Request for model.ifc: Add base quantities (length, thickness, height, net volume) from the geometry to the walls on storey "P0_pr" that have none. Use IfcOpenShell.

First a look at what the model holds.

```python
import ifcopenshell
import ifcopenshell.util.element
import ifcopenshell.util.unit

model = ifcopenshell.open("model.ifc")
print(model.schema)
for unit_type in ("LENGTHUNIT", "AREAUNIT", "VOLUMEUNIT"):
    print(unit_type, ifcopenshell.util.unit.calculate_unit_scale(model, unit_type))
storey = next(s for s in model.by_type("IfcBuildingStorey") if s.Name == "P0_pr")
walls = [e for e in ifcopenshell.util.element.get_decomposition(storey) if e.is_a("IfcWall")]
for e in sorted(walls, key=lambda e: e.id()):
    print(e.id(), e.is_a(), e.Name, list(ifcopenshell.util.element.get_psets(e, qtos_only=True)), sep=" | ")
```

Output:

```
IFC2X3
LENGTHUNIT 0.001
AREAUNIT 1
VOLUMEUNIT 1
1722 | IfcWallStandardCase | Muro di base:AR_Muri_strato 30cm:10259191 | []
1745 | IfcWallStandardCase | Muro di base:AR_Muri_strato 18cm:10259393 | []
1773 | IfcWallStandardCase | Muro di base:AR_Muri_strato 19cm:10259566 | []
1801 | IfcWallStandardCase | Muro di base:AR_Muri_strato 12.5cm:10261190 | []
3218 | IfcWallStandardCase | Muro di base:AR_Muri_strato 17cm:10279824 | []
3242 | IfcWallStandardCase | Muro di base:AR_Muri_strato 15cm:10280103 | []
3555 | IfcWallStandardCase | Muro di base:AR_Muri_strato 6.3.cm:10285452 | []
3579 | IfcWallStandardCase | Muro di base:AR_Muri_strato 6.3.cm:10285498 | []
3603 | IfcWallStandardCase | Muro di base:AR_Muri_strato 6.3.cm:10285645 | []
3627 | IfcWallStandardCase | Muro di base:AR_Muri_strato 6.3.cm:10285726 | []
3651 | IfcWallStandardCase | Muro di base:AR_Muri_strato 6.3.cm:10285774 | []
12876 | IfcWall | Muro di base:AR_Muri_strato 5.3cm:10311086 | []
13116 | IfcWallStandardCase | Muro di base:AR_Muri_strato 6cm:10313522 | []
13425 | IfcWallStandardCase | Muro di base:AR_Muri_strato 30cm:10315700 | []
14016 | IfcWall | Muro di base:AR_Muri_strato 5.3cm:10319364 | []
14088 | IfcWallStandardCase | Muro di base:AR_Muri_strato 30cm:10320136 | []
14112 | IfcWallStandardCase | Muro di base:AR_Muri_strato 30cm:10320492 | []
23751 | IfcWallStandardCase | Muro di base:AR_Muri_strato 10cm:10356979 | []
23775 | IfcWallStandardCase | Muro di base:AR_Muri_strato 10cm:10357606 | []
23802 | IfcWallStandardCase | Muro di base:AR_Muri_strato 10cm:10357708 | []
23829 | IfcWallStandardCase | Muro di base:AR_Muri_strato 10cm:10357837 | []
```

```python
import ifcopenshell
import ifcopenshell.api.pset
import ifcopenshell.geom
import ifcopenshell.util.element
import ifcopenshell.util.shape
import ifcopenshell.util.unit

model = ifcopenshell.open("model.ifc")
unit_scale = ifcopenshell.util.unit.calculate_unit_scale(model)
volume_scale = ifcopenshell.util.unit.calculate_unit_scale(model, "VOLUMEUNIT")
settings = ifcopenshell.geom.settings()

storey = next(s for s in model.by_type("IfcBuildingStorey") if s.Name == "P0_pr")
walls = [e for e in ifcopenshell.util.element.get_decomposition(storey) if e.is_a("IfcWall")]

for e in sorted(walls, key=lambda e: e.id()):
    if ifcopenshell.util.element.get_psets(e, qtos_only=True, should_inherit=False):
        continue
    # Geometry comes back in metres, in the element's own axes.
    shape = ifcopenshell.geom.create_shape(settings, e)
    values = {
        "Length": ifcopenshell.util.shape.get_x(shape.geometry) / unit_scale,
        "Width": ifcopenshell.util.shape.get_y(shape.geometry) / unit_scale,
        "Height": ifcopenshell.util.shape.get_z(shape.geometry) / unit_scale,
        "NetVolume": ifcopenshell.util.shape.get_volume(shape.geometry) / volume_scale,
    }
    qto = ifcopenshell.api.pset.add_qto(model, product=e, name="BaseQuantities")
    ifcopenshell.api.pset.edit_qto(model, qto=qto, properties=values)
    print(e.id(), {k: round(v, 3) for k, v in values.items()})

model.write("model_updated.ifc")
```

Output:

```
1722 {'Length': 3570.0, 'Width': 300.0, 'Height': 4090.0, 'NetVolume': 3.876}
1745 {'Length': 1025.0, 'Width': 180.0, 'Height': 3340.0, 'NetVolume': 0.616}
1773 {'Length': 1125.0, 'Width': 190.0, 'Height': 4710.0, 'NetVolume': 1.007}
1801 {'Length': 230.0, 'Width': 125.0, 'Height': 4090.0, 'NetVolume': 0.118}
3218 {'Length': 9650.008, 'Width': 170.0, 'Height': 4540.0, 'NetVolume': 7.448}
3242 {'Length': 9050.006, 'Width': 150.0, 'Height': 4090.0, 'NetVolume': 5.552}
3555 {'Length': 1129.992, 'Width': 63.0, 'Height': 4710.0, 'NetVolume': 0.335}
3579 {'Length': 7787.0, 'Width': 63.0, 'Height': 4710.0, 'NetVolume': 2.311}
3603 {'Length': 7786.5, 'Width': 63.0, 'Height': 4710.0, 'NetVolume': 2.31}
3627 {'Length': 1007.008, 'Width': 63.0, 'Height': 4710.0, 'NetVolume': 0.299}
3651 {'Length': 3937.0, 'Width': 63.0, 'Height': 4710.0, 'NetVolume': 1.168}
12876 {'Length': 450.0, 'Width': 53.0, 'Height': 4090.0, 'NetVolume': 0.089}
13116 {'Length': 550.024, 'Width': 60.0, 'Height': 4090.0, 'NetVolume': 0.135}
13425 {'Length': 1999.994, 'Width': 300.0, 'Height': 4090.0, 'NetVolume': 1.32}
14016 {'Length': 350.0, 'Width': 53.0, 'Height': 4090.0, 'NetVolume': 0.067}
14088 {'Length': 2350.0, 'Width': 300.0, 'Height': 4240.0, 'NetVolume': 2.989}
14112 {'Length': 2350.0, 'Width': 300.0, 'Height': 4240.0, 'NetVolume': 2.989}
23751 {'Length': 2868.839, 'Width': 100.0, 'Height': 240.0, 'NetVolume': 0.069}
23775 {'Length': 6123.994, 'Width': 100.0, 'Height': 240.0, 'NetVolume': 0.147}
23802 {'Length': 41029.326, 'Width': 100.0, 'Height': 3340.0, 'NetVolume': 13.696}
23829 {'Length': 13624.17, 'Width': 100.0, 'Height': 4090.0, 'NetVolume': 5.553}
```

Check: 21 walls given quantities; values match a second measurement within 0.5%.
